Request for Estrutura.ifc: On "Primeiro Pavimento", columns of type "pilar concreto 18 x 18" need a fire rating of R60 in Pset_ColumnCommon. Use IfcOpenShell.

First a look at what the model holds.

```python
import ifcopenshell
import ifcopenshell.util.element

model = ifcopenshell.open("Estrutura.ifc")
print(model.schema)
storey = next(s for s in model.by_type("IfcBuildingStorey") if s.Name == "Primeiro Pavimento")
columns = [e for e in ifcopenshell.util.element.get_decomposition(storey) if e.is_a("IfcColumn")]
seen = {}
for e in columns:
    element_type = ifcopenshell.util.element.get_type(e)
    key = (element_type.Name if element_type != e and element_type else None, ifcopenshell.util.element.get_pset(e, "Pset_ColumnCommon", "FireRating"))
    seen[key] = seen.get(key, 0) + 1
for (name, value), count in sorted(seen.items(), key=str):
    print(count, "x", name, "|", value)
```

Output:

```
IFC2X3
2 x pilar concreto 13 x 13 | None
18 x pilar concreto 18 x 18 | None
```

```python
import ifcopenshell
import ifcopenshell.api.pset
import ifcopenshell.util.element

model = ifcopenshell.open("Estrutura.ifc")

storey = next(s for s in model.by_type("IfcBuildingStorey") if s.Name == "Primeiro Pavimento")
columns = [e for e in ifcopenshell.util.element.get_decomposition(storey) if e.is_a("IfcColumn")]

count = 0
for e in columns:
    element_type = ifcopenshell.util.element.get_type(e)
    if element_type in (None, e) or element_type.Name != "pilar concreto 18 x 18":
        continue
    # add_pset returns the element's existing set when there is one.
    pset = ifcopenshell.api.pset.add_pset(model, product=e, name="Pset_ColumnCommon")
    ifcopenshell.api.pset.edit_pset(model, pset=pset, properties={"FireRating": "R60"})
    count += 1

print(count, "columns updated")

model.write("Estrutura_updated.ifc")
```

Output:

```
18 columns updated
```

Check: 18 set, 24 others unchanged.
